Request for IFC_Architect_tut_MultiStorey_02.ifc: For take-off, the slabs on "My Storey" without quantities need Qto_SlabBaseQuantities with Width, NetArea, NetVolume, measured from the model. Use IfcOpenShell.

First a look at what the model holds.

```python
import ifcopenshell
import ifcopenshell.util.element
import ifcopenshell.util.unit

model = ifcopenshell.open("IFC_Architect_tut_MultiStorey_02.ifc")
print(model.schema)
for unit_type in ("LENGTHUNIT", "AREAUNIT", "VOLUMEUNIT"):
    print(unit_type, ifcopenshell.util.unit.calculate_unit_scale(model, unit_type))
storey = next(s for s in model.by_type("IfcBuildingStorey") if s.Name == "My Storey")
slabs = [e for e in ifcopenshell.util.element.get_decomposition(storey) if e.is_a("IfcSlab")]
for e in sorted(slabs, key=lambda e: e.id()):
    print(e.id(), e.is_a(), e.Name, list(ifcopenshell.util.element.get_psets(e, qtos_only=True)), sep=" | ")
```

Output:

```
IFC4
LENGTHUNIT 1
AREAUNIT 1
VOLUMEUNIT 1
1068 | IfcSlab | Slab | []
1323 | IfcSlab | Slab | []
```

```python
import ifcopenshell
import ifcopenshell.api.pset
import ifcopenshell.geom
import ifcopenshell.util.element
import ifcopenshell.util.shape
import ifcopenshell.util.unit

model = ifcopenshell.open("IFC_Architect_tut_MultiStorey_02.ifc")
unit_scale = ifcopenshell.util.unit.calculate_unit_scale(model)
area_scale = ifcopenshell.util.unit.calculate_unit_scale(model, "AREAUNIT")
volume_scale = ifcopenshell.util.unit.calculate_unit_scale(model, "VOLUMEUNIT")
settings = ifcopenshell.geom.settings()

storey = next(s for s in model.by_type("IfcBuildingStorey") if s.Name == "My Storey")
slabs = [e for e in ifcopenshell.util.element.get_decomposition(storey) if e.is_a("IfcSlab")]

for e in sorted(slabs, key=lambda e: e.id()):
    if ifcopenshell.util.element.get_psets(e, qtos_only=True, should_inherit=False):
        continue
    # Geometry comes back in metres, in the element's own axes.
    shape = ifcopenshell.geom.create_shape(settings, e)
    values = {
        "Width": ifcopenshell.util.shape.get_z(shape.geometry) / unit_scale,
        "NetArea": ifcopenshell.util.shape.get_footprint_area(shape.geometry) / area_scale,
        "NetVolume": ifcopenshell.util.shape.get_volume(shape.geometry) / volume_scale,
    }
    qto = ifcopenshell.api.pset.add_qto(model, product=e, name="Qto_SlabBaseQuantities")
    ifcopenshell.api.pset.edit_qto(model, qto=qto, properties=values)
    print(e.id(), {k: round(v, 3) for k, v in values.items()})

model.write("IFC_Architect_tut_MultiStorey_02_v2.ifc")
```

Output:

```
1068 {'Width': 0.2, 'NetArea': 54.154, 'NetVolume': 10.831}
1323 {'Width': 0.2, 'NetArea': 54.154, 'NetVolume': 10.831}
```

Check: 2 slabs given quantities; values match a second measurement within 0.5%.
